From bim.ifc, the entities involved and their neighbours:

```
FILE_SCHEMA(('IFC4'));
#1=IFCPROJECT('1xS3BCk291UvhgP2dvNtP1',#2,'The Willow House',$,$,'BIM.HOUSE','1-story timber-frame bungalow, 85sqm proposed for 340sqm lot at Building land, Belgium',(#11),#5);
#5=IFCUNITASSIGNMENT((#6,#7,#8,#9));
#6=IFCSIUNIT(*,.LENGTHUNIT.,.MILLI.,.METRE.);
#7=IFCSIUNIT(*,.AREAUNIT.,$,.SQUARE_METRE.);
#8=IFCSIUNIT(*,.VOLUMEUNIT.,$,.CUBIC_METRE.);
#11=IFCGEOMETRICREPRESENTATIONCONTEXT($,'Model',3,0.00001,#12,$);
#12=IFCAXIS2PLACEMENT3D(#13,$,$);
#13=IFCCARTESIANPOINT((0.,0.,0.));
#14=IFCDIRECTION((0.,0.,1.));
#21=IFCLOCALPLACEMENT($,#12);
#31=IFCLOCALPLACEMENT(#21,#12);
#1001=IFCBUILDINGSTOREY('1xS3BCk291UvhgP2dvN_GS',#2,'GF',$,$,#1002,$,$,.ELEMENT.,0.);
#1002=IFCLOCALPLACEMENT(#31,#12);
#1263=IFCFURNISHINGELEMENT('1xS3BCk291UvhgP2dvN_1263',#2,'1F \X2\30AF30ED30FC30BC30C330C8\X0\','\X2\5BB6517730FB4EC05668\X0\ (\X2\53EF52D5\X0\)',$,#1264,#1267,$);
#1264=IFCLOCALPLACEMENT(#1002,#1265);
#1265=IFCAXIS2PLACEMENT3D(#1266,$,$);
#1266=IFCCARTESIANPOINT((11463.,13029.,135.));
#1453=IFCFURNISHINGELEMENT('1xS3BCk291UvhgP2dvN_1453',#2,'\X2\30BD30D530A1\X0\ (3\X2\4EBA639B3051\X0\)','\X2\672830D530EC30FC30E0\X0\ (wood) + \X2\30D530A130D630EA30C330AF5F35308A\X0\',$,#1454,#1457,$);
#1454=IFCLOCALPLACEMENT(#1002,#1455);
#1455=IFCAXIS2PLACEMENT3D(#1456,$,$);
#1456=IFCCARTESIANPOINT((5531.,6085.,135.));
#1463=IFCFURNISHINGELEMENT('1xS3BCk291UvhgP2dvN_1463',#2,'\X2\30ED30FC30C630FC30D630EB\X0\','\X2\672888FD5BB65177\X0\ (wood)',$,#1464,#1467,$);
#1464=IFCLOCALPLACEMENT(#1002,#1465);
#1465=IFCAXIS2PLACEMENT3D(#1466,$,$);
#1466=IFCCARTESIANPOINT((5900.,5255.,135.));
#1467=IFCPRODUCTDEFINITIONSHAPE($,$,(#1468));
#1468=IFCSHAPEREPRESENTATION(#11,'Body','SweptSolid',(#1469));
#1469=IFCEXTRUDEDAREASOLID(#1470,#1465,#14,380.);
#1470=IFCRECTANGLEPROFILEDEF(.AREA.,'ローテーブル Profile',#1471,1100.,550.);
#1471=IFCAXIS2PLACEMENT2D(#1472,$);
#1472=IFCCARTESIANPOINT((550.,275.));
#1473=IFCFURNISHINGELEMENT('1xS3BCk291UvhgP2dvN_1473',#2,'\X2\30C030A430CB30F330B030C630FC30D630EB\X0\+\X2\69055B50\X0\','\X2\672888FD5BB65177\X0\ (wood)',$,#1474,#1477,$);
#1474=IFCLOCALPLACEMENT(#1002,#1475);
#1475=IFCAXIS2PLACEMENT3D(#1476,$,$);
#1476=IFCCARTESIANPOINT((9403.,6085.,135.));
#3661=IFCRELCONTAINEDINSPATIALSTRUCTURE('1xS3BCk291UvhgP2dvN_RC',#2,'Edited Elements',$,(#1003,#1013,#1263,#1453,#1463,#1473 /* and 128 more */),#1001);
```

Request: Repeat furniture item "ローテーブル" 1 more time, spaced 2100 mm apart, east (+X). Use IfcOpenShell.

```python
import numpy as np
import ifcopenshell
import ifcopenshell.api.geometry
import ifcopenshell.api.root
import ifcopenshell.util.element
import ifcopenshell.util.placement
import ifcopenshell.util.unit

model = ifcopenshell.open("bim.ifc")
unit_scale = ifcopenshell.util.unit.calculate_unit_scale(model)


def reuse_history(source, copy):
    """copy_class also copies each property set's owner history, people and application; keep the originals."""
    for rel in copy.IsDefinedBy:
        if rel.is_a("IfcRelDefinesByProperties") and (history := rel.RelatingPropertyDefinition.OwnerHistory):
            rel.RelatingPropertyDefinition.OwnerHistory = source.OwnerHistory
            ifcopenshell.util.element.remove_deep2(model, history)


source = model.by_guid("1xS3BCk291UvhgP2dvN_1463")
base = ifcopenshell.util.placement.get_local_placement(source.ObjectPlacement)
step = np.array([1.0, 0.0, 0.0]) * 2.1 / unit_scale

for i in range(1, 2):
    copy = ifcopenshell.api.root.copy_class(model, product=source)
    copy.Representation = ifcopenshell.util.element.copy_deep(
        model, source.Representation, exclude=["IfcGeometricRepresentationContext", "IfcRepresentationMap"]
    )
    reuse_history(source, copy)
    matrix = base.copy()
    matrix[:3, 3] += i * step
    print("added at", matrix[:3, 3].round(3) + 0.0)
    ifcopenshell.api.geometry.edit_object_placement(model, product=copy, matrix=matrix, is_si=False)

model.write("bim_edited.ifc")
```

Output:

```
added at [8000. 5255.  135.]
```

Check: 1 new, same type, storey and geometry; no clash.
